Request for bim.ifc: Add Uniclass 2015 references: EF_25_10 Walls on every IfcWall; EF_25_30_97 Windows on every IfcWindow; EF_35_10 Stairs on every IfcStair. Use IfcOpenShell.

First a look at what the model holds.

```python
import ifcopenshell

model = ifcopenshell.open("bim.ifc")
print(model.schema)
print("classifications:", [c.Name for c in model.by_type("IfcClassification")])
for ifc_class in ("IfcDoor", "IfcRoof", "IfcStair", "IfcWall", "IfcWindow"):
    print(ifc_class, len(model.by_type(ifc_class)))
```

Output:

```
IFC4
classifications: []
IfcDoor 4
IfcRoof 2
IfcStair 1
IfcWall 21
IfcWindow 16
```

```python
import ifcopenshell
import ifcopenshell.api.classification

model = ifcopenshell.open("bim.ifc")

system = ifcopenshell.api.classification.add_classification(model, classification="Uniclass 2015")

codes = {
    "IfcWall": ("EF_25_10", "Walls"),
    "IfcWindow": ("EF_25_30_97", "Windows"),
    "IfcStair": ("EF_35_10", "Stairs"),
}
for ifc_class, (code, name) in codes.items():
    products = model.by_type(ifc_class)
    ifcopenshell.api.classification.add_reference(
        model, products=products, classification=system, identification=code, name=name
    )
    print(code, len(products))

model.write("bim-out.ifc")
```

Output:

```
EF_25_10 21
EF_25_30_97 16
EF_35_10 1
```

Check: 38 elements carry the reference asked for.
